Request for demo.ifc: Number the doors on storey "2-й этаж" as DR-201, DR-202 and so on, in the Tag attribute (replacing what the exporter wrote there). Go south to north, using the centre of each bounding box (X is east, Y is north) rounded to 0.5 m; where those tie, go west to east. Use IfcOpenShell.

First a look at what the model holds.

```python
import ifcopenshell
import ifcopenshell.util.element
import ifcopenshell.util.placement

model = ifcopenshell.open("demo.ifc")
print(model.schema)
storey = next(s for s in model.by_type("IfcBuildingStorey") if s.Name == "2-й этаж")
doors = [e for e in ifcopenshell.util.element.get_decomposition(storey) if e.is_a("IfcDoor")]
for e in sorted(doors, key=lambda e: e.id()):
    origin = ifcopenshell.util.placement.get_local_placement(e.ObjectPlacement)[:3, 3]
    print(e.id(), e.Tag, e.Name, origin.round(2) + 0.0, sep=" | ")
```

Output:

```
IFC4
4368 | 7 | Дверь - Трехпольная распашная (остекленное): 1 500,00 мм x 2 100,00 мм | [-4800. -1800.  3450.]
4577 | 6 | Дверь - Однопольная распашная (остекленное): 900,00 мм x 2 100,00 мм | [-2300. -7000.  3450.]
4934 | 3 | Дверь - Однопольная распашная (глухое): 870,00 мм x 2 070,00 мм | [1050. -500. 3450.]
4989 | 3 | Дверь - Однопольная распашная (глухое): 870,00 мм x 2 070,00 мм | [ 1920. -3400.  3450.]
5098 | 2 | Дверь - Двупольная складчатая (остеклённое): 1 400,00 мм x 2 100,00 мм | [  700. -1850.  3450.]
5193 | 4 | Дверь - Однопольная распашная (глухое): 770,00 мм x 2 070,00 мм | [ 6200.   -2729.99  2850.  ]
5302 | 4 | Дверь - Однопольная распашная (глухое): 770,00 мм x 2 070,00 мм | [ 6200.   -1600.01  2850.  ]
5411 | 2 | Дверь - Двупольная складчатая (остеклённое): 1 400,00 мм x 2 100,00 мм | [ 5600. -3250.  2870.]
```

```python
import ifcopenshell
import ifcopenshell.geom
import ifcopenshell.util.element
import ifcopenshell.util.shape

model = ifcopenshell.open("demo.ifc")
settings = ifcopenshell.geom.settings()
settings.set("use-world-coords", True)


def centre(element):
    shape = ifcopenshell.geom.create_shape(settings, element)
    return ifcopenshell.util.shape.get_bbox_centroid(shape.geometry)


storey = next(s for s in model.by_type("IfcBuildingStorey") if s.Name == "2-й этаж")
doors = [e for e in ifcopenshell.util.element.get_decomposition(storey) if e.is_a("IfcDoor")]

# Insertion points can sit at a corner or the storey origin, so sort by the geometry (in metres).
centres = {e: centre(e) for e in doors}
doors.sort(key=lambda e: (round(centres[e][1] / 0.5), centres[e][0]))

for i, e in enumerate(doors, start=1):
    number = f"DR-2{i:02d}"
    e.Tag = number
    print(e.id(), number)

model.write("demo_v2.ifc")
```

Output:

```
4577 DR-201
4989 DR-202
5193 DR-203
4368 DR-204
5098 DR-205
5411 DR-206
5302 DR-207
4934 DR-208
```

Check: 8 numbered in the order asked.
